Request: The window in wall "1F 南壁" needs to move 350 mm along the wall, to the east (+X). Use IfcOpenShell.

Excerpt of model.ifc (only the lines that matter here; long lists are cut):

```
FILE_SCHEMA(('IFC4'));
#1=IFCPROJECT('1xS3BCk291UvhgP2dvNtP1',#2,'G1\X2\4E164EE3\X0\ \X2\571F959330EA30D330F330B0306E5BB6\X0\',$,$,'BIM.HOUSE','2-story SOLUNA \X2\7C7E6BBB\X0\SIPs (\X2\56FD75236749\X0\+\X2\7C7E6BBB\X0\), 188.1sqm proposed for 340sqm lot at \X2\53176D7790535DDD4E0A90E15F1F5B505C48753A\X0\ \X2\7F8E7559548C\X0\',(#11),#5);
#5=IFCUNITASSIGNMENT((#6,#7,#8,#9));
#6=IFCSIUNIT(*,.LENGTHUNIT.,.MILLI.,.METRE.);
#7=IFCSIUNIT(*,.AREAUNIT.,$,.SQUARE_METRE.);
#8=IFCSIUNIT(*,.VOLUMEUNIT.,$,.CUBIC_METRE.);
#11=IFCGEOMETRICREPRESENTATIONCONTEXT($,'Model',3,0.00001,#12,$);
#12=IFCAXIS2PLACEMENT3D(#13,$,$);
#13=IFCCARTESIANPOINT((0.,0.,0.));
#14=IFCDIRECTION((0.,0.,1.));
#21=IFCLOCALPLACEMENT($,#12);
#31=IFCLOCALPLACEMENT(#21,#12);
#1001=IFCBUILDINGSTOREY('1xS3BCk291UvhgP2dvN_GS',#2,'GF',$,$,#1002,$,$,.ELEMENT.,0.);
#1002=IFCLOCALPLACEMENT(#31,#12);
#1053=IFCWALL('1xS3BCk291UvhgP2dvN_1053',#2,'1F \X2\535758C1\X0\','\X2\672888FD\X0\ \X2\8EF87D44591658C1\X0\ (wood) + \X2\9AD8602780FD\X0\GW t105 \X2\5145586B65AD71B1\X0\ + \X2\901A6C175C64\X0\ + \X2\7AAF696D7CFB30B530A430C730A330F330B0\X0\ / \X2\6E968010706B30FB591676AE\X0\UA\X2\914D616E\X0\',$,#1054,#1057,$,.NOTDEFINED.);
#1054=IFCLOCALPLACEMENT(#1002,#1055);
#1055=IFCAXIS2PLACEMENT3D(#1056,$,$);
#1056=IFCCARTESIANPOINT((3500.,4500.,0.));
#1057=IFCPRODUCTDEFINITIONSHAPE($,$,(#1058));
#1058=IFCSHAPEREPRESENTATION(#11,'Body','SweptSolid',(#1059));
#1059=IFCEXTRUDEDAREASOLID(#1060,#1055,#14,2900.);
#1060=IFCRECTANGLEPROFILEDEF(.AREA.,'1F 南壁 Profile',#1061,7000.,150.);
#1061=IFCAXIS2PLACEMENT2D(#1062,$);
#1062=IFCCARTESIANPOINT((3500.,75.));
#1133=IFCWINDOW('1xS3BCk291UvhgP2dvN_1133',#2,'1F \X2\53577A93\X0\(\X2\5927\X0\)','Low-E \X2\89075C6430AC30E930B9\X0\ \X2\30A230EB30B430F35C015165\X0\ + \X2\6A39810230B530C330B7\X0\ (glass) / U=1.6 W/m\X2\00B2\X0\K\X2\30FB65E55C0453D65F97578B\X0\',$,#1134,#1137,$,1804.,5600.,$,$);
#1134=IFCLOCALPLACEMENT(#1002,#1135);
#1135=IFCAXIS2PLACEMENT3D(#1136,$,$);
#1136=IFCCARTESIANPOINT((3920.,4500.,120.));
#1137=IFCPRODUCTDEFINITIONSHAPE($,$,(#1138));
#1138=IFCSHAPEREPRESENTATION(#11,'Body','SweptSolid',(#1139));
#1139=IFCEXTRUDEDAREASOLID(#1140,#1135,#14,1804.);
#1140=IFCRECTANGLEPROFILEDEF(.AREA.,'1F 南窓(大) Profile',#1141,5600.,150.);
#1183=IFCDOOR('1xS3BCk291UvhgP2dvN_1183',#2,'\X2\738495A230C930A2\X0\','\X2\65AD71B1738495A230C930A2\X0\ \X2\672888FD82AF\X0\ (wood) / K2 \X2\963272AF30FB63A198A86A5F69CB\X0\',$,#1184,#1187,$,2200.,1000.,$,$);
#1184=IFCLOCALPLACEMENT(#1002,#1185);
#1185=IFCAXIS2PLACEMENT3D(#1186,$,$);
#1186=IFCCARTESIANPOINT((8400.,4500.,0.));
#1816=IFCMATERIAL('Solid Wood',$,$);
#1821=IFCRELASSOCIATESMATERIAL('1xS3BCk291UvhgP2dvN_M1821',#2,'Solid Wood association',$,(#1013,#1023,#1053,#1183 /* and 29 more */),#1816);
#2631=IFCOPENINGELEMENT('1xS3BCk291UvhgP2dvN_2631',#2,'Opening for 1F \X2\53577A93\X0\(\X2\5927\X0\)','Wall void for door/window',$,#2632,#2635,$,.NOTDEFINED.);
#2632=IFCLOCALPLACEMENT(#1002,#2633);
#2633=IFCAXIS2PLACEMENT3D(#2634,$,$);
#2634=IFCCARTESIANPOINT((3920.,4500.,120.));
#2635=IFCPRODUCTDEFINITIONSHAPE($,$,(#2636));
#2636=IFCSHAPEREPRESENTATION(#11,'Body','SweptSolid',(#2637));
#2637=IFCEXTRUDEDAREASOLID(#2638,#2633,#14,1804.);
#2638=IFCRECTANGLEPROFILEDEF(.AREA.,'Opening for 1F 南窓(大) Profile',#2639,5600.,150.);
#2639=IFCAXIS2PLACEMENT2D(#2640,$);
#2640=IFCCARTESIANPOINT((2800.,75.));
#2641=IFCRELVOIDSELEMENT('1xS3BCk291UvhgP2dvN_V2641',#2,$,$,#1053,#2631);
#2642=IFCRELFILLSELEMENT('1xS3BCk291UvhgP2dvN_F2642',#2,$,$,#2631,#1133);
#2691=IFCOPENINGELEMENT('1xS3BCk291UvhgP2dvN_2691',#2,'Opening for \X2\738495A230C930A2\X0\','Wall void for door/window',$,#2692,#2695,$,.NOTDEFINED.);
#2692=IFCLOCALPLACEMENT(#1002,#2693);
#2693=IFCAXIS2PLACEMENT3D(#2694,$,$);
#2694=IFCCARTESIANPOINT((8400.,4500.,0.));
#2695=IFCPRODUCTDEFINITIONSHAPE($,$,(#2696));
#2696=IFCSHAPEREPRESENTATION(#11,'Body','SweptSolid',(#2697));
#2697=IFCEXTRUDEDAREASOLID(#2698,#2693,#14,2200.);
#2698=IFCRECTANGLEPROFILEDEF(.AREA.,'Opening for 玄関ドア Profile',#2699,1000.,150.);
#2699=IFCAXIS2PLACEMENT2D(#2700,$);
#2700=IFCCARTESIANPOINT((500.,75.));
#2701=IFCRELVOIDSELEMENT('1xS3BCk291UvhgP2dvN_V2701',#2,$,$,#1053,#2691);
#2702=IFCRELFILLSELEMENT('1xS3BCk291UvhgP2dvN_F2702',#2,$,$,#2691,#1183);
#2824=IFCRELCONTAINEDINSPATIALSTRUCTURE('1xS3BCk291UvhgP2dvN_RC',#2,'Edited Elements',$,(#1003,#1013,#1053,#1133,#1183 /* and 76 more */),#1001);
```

```python
import ifcopenshell
import ifcopenshell.api.geometry
import ifcopenshell.util.placement

model = ifcopenshell.open("model.ifc")

window = model.by_guid("1xS3BCk291UvhgP2dvN_1133")
opening = window.FillsVoids[0].RelatingOpeningElement
wall = opening.VoidsElements[0].RelatingBuildingElement

wall_matrix = ifcopenshell.util.placement.get_local_placement(wall.ObjectPlacement)
shift = wall_matrix[:3, 0] * 350.0
before = ifcopenshell.util.placement.get_local_placement(window.ObjectPlacement)[:3, 3].copy()

# The window is not placed relative to its opening, so move both.
for product in (opening, window):
    matrix = ifcopenshell.util.placement.get_local_placement(product.ObjectPlacement)
    matrix[:3, 3] += shift
    ifcopenshell.api.geometry.edit_object_placement(model, product=product, matrix=matrix, is_si=False)

after = ifcopenshell.util.placement.get_local_placement(window.ObjectPlacement)[:3, 3]
print("window moved by", (after - before).round(3) + 0.0)

model.write("model_v2.ifc")
```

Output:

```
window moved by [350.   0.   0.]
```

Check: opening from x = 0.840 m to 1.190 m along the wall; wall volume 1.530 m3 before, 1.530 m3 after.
